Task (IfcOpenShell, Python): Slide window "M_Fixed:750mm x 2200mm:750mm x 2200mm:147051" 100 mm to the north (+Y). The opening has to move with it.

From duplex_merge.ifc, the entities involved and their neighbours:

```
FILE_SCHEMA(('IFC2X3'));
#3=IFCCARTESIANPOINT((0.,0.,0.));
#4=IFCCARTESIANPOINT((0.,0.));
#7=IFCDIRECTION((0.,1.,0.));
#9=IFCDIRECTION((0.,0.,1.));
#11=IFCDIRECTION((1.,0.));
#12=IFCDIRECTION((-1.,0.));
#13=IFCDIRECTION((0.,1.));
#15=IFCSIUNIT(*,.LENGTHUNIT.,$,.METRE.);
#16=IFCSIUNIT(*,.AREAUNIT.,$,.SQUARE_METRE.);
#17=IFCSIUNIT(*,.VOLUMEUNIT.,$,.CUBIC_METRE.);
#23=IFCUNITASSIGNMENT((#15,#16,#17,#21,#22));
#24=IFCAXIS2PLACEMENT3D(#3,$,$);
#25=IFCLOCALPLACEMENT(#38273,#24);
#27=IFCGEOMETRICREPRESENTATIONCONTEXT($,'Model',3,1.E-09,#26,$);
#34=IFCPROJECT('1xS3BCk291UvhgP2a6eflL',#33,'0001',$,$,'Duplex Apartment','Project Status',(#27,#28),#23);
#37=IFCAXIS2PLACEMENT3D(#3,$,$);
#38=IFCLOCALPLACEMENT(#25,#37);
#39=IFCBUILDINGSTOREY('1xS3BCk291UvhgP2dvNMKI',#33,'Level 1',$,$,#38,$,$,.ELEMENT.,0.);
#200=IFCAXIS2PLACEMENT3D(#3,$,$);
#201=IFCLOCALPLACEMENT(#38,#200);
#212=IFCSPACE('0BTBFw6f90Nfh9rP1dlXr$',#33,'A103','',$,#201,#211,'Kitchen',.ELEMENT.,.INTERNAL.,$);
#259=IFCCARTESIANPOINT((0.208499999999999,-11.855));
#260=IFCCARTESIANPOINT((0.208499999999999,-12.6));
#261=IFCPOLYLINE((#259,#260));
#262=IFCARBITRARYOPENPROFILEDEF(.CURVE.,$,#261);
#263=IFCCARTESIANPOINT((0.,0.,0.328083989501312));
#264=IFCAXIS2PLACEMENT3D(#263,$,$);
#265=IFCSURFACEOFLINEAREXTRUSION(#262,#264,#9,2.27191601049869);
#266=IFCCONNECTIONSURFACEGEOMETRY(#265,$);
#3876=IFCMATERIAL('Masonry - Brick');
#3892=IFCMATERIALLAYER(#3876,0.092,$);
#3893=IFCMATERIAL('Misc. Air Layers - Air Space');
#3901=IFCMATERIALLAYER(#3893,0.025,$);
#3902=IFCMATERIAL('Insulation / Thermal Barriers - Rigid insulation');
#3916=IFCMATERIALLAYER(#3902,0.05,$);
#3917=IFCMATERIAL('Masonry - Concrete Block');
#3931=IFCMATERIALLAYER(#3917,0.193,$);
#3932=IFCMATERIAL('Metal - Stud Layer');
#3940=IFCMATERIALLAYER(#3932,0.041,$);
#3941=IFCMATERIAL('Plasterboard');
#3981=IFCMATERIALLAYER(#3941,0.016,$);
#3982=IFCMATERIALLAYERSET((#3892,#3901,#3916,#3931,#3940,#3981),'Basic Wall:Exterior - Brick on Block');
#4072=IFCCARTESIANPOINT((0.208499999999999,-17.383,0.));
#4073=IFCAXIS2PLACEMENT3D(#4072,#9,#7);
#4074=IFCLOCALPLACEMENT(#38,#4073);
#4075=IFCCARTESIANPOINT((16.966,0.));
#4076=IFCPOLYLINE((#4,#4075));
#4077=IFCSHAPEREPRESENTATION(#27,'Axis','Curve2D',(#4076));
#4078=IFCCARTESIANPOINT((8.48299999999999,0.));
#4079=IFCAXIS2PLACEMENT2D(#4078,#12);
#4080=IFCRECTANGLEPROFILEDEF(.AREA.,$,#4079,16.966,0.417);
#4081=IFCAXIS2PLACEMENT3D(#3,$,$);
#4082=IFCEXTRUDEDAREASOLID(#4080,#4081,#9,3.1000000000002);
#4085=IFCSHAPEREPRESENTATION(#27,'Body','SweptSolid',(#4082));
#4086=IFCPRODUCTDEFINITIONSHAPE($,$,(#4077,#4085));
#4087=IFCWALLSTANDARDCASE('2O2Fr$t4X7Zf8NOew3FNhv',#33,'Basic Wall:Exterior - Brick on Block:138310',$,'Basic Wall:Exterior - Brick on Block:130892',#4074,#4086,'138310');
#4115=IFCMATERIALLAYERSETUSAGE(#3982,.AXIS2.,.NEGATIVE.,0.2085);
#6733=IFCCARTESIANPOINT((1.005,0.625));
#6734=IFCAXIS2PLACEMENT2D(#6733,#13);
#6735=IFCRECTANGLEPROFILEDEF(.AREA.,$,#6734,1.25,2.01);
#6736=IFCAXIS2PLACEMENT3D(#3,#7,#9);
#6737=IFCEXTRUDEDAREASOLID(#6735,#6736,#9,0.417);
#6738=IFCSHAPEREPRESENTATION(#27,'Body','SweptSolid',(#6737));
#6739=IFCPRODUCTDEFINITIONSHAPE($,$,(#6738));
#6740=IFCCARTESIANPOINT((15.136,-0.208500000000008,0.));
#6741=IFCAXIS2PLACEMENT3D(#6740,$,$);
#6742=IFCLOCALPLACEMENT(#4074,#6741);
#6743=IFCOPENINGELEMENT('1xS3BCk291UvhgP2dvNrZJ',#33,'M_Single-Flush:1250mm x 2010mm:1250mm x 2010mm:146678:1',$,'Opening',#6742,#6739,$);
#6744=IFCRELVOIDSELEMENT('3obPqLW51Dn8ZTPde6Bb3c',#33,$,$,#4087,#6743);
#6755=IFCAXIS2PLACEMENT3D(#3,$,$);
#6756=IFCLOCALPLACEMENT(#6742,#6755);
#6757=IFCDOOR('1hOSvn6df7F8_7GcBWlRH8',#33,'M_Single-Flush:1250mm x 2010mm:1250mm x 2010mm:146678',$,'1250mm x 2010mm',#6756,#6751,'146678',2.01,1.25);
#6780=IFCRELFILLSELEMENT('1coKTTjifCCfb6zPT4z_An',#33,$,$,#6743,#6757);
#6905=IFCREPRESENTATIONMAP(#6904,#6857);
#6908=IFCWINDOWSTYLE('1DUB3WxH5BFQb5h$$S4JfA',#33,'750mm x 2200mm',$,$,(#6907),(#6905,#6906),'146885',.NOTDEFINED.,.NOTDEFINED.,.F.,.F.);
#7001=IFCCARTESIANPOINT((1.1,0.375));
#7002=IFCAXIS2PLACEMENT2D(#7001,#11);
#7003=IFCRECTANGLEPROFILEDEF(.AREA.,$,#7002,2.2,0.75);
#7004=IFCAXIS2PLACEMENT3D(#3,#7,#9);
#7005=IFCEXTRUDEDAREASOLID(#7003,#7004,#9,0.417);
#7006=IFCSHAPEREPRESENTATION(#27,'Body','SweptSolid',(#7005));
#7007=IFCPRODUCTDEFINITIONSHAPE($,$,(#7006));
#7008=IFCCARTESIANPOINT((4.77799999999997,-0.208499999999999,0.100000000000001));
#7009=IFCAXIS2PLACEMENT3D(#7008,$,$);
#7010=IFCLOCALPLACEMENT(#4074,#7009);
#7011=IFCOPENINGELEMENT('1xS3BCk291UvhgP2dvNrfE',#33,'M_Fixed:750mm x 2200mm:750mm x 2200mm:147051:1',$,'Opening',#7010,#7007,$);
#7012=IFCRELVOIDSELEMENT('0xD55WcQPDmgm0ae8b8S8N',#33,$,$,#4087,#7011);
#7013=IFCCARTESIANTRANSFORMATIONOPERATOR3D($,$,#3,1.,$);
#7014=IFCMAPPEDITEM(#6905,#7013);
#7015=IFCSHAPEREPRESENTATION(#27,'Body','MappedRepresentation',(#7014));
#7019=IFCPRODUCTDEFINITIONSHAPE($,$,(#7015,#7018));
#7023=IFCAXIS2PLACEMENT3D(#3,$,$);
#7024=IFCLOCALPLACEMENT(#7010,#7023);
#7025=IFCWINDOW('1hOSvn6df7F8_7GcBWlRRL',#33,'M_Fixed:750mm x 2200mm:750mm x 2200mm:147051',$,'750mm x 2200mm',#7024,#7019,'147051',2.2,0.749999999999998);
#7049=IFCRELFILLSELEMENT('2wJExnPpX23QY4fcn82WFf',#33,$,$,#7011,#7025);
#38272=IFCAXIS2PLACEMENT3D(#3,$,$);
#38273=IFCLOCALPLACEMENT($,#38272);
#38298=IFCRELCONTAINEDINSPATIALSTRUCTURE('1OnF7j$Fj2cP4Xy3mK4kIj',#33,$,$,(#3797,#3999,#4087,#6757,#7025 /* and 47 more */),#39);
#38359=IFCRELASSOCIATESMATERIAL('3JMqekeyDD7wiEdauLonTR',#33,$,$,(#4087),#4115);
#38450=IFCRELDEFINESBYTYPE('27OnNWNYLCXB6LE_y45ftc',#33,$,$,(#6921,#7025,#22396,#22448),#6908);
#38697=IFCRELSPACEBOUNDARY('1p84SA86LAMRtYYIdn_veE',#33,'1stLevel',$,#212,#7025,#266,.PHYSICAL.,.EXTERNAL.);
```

```python
import numpy as np
import ifcopenshell
import ifcopenshell.api.geometry
import ifcopenshell.util.placement
import ifcopenshell.util.unit

model = ifcopenshell.open("duplex_merge.ifc")
unit_scale = ifcopenshell.util.unit.calculate_unit_scale(model)

window = model.by_guid("1hOSvn6df7F8_7GcBWlRRL")
opening = window.FillsVoids[0].RelatingOpeningElement
wall = opening.VoidsElements[0].RelatingBuildingElement

wall_matrix = ifcopenshell.util.placement.get_local_placement(wall.ObjectPlacement)
shift = wall_matrix[:3, 0] * 0.1 / unit_scale
before = ifcopenshell.util.placement.get_local_placement(window.ObjectPlacement)[:3, 3].copy()

# The window is placed relative to its opening, so it follows when the opening moves.
matrix = ifcopenshell.util.placement.get_local_placement(opening.ObjectPlacement)
matrix[:3, 3] += shift
ifcopenshell.api.geometry.edit_object_placement(
    model, product=opening, matrix=matrix, is_si=False, should_transform_children=True
)

# Space boundary surfaces are stored in each space's coordinates; move them too.
for rel in window.ProvidesBoundaries:
    if not rel.ConnectionGeometry:
        continue
    surface = rel.ConnectionGeometry.SurfaceOnRelatingElement
    space_matrix = ifcopenshell.util.placement.get_local_placement(rel.RelatingSpace.ObjectPlacement)
    point = np.array(surface.Position.Location.Coordinates) + space_matrix[:3, :3].T @ shift
    surface.Position = model.createIfcAxis2Placement3D(
        model.createIfcCartesianPoint(point.tolist()), surface.Position.Axis, surface.Position.RefDirection
    )

after = ifcopenshell.util.placement.get_local_placement(window.ObjectPlacement)[:3, 3]
print("window moved by", (after - before).round(3) + 0.0)

model.write("duplex_merge_rev.ifc")
```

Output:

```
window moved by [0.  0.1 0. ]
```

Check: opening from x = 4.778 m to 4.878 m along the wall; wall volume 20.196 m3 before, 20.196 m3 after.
